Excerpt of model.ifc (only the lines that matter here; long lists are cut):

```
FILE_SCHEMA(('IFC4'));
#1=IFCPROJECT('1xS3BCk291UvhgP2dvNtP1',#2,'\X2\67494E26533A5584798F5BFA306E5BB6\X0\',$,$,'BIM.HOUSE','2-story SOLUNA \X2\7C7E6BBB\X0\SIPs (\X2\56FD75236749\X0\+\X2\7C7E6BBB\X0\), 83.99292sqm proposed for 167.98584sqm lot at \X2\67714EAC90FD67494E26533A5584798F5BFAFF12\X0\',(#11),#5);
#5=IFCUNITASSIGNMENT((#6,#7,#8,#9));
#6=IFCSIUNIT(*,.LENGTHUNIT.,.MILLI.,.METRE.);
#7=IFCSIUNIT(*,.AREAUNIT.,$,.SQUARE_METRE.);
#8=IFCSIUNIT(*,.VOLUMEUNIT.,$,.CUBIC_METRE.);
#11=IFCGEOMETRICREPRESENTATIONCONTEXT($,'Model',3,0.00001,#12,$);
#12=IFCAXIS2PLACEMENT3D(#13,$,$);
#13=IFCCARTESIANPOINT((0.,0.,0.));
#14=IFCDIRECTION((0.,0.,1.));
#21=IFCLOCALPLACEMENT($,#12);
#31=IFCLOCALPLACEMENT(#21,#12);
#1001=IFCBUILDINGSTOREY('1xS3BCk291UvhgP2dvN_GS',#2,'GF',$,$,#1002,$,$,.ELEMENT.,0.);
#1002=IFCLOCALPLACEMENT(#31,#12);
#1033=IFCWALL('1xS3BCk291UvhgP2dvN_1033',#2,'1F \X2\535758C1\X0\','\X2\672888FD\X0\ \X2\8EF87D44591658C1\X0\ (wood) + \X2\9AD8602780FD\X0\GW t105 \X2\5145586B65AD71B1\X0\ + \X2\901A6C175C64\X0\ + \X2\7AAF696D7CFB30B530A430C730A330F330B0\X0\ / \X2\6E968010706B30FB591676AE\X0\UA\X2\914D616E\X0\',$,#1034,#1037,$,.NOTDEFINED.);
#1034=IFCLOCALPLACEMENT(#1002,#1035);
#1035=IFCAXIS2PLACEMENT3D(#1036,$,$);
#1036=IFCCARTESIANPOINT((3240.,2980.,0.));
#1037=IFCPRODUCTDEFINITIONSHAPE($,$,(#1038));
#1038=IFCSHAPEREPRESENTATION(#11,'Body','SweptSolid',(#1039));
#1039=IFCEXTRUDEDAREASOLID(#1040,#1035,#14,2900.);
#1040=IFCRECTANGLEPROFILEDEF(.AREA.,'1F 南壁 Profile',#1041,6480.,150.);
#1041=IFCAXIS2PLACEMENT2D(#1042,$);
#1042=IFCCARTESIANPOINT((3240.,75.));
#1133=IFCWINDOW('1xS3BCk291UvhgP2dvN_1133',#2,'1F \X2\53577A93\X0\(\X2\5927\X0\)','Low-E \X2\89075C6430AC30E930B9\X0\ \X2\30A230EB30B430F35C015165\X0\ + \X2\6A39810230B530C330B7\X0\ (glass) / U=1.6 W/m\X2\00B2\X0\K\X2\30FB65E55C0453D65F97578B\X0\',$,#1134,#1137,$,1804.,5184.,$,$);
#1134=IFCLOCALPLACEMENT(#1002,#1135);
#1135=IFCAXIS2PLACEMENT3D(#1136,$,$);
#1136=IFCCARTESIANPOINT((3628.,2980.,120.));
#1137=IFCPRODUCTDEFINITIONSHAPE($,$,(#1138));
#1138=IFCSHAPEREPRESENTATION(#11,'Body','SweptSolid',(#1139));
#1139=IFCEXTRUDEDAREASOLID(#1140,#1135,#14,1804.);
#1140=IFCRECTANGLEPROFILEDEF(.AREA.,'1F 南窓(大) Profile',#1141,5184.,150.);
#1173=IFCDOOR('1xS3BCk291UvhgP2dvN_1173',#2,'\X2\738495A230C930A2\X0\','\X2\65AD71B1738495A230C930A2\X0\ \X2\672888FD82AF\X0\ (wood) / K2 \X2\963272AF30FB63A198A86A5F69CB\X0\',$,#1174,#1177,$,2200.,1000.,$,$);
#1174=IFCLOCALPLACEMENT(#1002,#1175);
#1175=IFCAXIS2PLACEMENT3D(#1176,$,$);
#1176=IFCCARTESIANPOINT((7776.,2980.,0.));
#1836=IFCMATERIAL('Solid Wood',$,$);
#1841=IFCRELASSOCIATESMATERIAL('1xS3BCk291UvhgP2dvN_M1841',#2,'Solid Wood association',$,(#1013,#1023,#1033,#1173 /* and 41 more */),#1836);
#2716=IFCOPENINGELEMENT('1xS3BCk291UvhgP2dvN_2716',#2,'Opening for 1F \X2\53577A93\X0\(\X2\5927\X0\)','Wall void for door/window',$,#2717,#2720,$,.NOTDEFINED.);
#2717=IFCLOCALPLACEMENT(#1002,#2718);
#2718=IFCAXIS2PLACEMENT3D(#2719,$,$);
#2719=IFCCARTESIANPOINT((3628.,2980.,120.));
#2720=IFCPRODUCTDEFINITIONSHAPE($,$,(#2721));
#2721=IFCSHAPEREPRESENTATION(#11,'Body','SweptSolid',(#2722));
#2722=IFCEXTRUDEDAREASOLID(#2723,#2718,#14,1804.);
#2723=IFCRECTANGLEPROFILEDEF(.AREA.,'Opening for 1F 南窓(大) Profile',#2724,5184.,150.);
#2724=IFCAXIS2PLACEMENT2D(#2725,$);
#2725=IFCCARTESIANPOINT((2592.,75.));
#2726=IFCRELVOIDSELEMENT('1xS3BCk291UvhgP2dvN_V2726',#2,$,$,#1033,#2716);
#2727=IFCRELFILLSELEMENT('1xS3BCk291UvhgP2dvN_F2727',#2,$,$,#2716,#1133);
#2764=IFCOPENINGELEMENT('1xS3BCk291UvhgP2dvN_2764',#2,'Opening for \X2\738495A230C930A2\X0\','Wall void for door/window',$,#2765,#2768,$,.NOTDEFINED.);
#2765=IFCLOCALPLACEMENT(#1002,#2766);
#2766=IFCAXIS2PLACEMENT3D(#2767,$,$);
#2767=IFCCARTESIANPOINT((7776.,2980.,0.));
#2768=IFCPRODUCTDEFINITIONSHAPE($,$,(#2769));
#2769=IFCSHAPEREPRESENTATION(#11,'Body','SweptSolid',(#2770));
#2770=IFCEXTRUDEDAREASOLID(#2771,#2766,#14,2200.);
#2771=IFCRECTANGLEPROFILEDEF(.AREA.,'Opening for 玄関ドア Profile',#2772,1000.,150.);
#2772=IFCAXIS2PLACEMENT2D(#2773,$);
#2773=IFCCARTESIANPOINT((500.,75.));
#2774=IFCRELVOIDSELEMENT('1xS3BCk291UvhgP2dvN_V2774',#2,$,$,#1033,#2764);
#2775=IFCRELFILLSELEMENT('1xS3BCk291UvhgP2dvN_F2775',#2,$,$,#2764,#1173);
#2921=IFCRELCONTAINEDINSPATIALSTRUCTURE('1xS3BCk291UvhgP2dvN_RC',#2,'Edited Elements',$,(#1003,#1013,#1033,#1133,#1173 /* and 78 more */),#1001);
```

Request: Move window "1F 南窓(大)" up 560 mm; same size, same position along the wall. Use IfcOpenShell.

```python
import numpy as np
import ifcopenshell
import ifcopenshell.api.geometry
import ifcopenshell.util.placement
import ifcopenshell.util.unit

model = ifcopenshell.open("model.ifc")
unit_scale = ifcopenshell.util.unit.calculate_unit_scale(model)

window = model.by_id(1133)
opening = window.FillsVoids[0].RelatingOpeningElement
dz = 0.56 / unit_scale

shift = np.array([0.0, 0.0, dz])
# The window is not placed relative to its opening, so move both.
for product in (opening, window):
    matrix = ifcopenshell.util.placement.get_local_placement(product.ObjectPlacement)
    matrix[:3, 3] += shift
    ifcopenshell.api.geometry.edit_object_placement(model, product=product, matrix=matrix, is_si=False)

print(f"moved by {dz * unit_scale:+.3f} m")

model.write("model_updated.ifc")
```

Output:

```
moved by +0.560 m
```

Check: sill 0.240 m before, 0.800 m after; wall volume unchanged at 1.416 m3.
